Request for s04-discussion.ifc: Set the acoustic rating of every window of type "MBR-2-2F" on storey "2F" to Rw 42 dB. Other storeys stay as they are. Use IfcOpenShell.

First a look at what the model holds.

```python
import ifcopenshell
import ifcopenshell.util.element

model = ifcopenshell.open("s04-discussion.ifc")
print(model.schema)
storey = next(s for s in model.by_type("IfcBuildingStorey") if s.Name == "2F")
windows = [e for e in ifcopenshell.util.element.get_decomposition(storey) if e.is_a("IfcWindow")]
seen = {}
for e in windows:
    element_type = ifcopenshell.util.element.get_type(e)
    key = (element_type.Name if element_type != e and element_type else None, ifcopenshell.util.element.get_pset(e, "Pset_WindowCommon", "AcousticRating"))
    seen[key] = seen.get(key, 0) + 1
for (name, value), count in sorted(seen.items(), key=str):
    print(count, "x", name, "|", value)
```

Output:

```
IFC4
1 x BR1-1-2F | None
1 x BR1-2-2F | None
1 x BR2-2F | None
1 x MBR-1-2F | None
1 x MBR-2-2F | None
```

```python
import ifcopenshell
import ifcopenshell.api.pset
import ifcopenshell.util.element

model = ifcopenshell.open("s04-discussion.ifc")

storey = next(s for s in model.by_type("IfcBuildingStorey") if s.Name == "2F")
windows = [e for e in ifcopenshell.util.element.get_decomposition(storey) if e.is_a("IfcWindow")]

count = 0
for e in windows:
    element_type = ifcopenshell.util.element.get_type(e)
    if element_type in (None, e) or element_type.Name != "MBR-2-2F":
        continue
    # add_pset returns the element's existing set when there is one.
    pset = ifcopenshell.api.pset.add_pset(model, product=e, name="Pset_WindowCommon")
    ifcopenshell.api.pset.edit_pset(model, pset=pset, properties={"AcousticRating": "Rw 42 dB"})
    count += 1

print(count, "windows updated")

model.write("s04-discussion_rev.ifc")
```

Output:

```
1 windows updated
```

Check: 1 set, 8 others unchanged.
